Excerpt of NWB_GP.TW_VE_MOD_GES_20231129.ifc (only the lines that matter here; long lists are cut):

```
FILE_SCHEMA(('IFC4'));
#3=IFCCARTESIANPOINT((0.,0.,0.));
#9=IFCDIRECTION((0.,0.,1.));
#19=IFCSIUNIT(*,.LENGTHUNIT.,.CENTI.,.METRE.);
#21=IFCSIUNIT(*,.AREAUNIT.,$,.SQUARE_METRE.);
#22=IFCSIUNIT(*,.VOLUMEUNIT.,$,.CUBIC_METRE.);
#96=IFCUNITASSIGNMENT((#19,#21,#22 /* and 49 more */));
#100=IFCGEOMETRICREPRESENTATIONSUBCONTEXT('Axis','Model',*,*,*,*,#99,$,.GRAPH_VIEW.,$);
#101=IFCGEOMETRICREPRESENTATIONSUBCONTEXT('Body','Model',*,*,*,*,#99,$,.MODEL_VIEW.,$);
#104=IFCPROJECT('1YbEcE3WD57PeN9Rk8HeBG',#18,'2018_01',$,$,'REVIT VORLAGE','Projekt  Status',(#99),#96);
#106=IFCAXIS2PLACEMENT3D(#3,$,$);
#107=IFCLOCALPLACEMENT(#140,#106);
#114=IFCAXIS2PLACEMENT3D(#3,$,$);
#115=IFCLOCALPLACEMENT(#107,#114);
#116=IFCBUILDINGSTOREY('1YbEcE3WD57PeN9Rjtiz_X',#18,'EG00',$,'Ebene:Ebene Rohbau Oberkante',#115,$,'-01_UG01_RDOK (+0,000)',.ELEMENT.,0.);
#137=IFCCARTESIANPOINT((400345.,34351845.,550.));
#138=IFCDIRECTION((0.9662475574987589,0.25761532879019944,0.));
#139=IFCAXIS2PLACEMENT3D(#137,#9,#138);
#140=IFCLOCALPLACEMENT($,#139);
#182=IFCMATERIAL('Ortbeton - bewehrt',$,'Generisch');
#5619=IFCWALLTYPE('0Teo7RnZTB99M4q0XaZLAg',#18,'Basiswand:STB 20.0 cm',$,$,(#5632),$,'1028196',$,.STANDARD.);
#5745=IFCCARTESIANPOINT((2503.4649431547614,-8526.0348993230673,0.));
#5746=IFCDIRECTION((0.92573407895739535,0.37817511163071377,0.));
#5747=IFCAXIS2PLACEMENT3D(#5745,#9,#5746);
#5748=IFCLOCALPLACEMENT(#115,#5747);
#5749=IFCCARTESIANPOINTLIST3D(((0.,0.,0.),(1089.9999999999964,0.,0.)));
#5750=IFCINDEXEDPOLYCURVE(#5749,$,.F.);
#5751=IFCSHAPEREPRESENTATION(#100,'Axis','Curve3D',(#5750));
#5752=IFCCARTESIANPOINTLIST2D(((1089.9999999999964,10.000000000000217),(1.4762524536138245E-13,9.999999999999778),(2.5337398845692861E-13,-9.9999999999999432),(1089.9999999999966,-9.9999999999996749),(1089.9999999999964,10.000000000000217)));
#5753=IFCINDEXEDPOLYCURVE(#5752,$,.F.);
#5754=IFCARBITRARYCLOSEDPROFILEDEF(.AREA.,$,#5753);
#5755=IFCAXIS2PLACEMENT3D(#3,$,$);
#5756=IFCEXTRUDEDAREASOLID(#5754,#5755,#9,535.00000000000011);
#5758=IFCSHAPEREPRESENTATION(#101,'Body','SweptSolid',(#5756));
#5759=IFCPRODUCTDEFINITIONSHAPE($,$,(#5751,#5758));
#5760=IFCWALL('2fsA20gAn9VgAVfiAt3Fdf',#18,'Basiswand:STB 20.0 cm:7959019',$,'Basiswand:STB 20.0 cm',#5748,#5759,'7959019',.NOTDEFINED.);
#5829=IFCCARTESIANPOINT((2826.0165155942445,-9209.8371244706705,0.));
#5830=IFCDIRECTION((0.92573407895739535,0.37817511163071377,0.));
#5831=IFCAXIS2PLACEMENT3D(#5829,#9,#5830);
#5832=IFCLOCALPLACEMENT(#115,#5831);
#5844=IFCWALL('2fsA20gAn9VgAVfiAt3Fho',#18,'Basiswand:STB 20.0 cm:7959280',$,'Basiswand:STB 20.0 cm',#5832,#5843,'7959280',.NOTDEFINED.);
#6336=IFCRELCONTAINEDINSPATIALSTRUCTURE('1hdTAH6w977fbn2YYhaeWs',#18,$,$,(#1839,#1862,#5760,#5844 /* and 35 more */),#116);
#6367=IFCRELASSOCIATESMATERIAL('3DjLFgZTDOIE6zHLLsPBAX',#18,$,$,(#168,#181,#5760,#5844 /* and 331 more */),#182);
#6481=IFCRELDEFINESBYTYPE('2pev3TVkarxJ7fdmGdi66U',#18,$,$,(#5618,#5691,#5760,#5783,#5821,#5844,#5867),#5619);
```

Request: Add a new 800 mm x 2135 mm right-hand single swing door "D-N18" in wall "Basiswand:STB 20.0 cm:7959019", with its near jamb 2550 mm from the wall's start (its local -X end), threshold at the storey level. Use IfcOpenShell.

```python
import numpy as np
import ifcopenshell
import ifcopenshell.api.feature
import ifcopenshell.api.geometry
import ifcopenshell.api.root
import ifcopenshell.api.spatial
import ifcopenshell.geom
import ifcopenshell.util.element
import ifcopenshell.util.placement
import ifcopenshell.util.representation
import ifcopenshell.util.shape
import ifcopenshell.util.unit

model = ifcopenshell.open("NWB_GP.TW_VE_MOD_GES_20231129.ifc")
unit_scale = ifcopenshell.util.unit.calculate_unit_scale(model)
settings = ifcopenshell.geom.settings()


def volume(element):
    """Net volume in cubic metres, openings subtracted."""
    shape = ifcopenshell.geom.create_shape(settings, element)
    return ifcopenshell.util.shape.get_volume(shape.geometry)


wall = model.by_guid("2fsA20gAn9VgAVfiAt3Fdf")
storey = ifcopenshell.util.element.get_container(wall, ifc_class="IfcBuildingStorey")
context = ifcopenshell.util.representation.get_context(model, "Model", "Body", "MODEL_VIEW")
before = volume(wall)

width, height, from_end, sill = 0.8, 2.135, 2.55, 0.0  # metres

# The wall runs along its own X axis, and the end named is its -X end.
wall_shape = ifcopenshell.geom.create_shape(settings, wall)
x, y, z = ifcopenshell.util.shape.get_vertices(wall_shape.geometry).T
start = x.min() + from_end
face, thickness = float(y.min()), float(y.max() - y.min())
wall_matrix = ifcopenshell.util.placement.get_local_placement(wall.ObjectPlacement)
level = ifcopenshell.util.placement.get_local_placement(storey.ObjectPlacement)[2, 3]


def in_wall(x, y):
    """Placement at x, y metres in the wall's axes, at sill height."""
    matrix = wall_matrix.copy()
    matrix[:, 3] = wall_matrix @ np.array([x / unit_scale, y / unit_scale, 0.0, 1.0])
    matrix[2, 3] = level + sill / unit_scale
    return matrix


# Opening: a box that overshoots both wall faces by 50 mm.
opening = ifcopenshell.api.root.create_entity(model, ifc_class="IfcOpeningElement", predefined_type="OPENING")
box = ifcopenshell.api.geometry.add_wall_representation(
    model, context=context, length=width, height=height, thickness=thickness + 0.1
)
ifcopenshell.api.geometry.assign_representation(model, product=opening, representation=box)
ifcopenshell.api.geometry.edit_object_placement(model, product=opening, matrix=in_wall(start, face - 0.05), is_si=False)
ifcopenshell.api.feature.add_feature(model, feature=opening, element=wall)

door = ifcopenshell.api.root.create_entity(model, ifc_class="IfcDoor", name="D-N18", predefined_type="DOOR")
door.OverallWidth, door.OverallHeight = width / unit_scale, height / unit_scale
door.OperationType = "SINGLE_SWING_RIGHT"
body = ifcopenshell.api.geometry.add_door_representation(
    model,
    context=context,
    overall_width=door.OverallWidth,
    overall_height=door.OverallHeight,
    operation_type="SINGLE_SWING_RIGHT",
    lining_properties={"LiningDepth": thickness / unit_scale, "ThresholdDepth": thickness / unit_scale},
)
ifcopenshell.api.geometry.assign_representation(model, product=door, representation=body)
ifcopenshell.api.spatial.assign_container(model, products=[door], relating_structure=storey)
ifcopenshell.api.feature.add_filling(model, opening=opening, element=door)

# The lining spans the wall, so the door starts at the wall face.
ifcopenshell.api.geometry.edit_object_placement(model, product=door, matrix=in_wall(start, face), is_si=False)

after = volume(wall)

print(f"wall volume {before:.3f} -> {after:.3f} m3")

model.write("NWB_GP.TW_VE_MOD_GES_20231129-out.ifc")
```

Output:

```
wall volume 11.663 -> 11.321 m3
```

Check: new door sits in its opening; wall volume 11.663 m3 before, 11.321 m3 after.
